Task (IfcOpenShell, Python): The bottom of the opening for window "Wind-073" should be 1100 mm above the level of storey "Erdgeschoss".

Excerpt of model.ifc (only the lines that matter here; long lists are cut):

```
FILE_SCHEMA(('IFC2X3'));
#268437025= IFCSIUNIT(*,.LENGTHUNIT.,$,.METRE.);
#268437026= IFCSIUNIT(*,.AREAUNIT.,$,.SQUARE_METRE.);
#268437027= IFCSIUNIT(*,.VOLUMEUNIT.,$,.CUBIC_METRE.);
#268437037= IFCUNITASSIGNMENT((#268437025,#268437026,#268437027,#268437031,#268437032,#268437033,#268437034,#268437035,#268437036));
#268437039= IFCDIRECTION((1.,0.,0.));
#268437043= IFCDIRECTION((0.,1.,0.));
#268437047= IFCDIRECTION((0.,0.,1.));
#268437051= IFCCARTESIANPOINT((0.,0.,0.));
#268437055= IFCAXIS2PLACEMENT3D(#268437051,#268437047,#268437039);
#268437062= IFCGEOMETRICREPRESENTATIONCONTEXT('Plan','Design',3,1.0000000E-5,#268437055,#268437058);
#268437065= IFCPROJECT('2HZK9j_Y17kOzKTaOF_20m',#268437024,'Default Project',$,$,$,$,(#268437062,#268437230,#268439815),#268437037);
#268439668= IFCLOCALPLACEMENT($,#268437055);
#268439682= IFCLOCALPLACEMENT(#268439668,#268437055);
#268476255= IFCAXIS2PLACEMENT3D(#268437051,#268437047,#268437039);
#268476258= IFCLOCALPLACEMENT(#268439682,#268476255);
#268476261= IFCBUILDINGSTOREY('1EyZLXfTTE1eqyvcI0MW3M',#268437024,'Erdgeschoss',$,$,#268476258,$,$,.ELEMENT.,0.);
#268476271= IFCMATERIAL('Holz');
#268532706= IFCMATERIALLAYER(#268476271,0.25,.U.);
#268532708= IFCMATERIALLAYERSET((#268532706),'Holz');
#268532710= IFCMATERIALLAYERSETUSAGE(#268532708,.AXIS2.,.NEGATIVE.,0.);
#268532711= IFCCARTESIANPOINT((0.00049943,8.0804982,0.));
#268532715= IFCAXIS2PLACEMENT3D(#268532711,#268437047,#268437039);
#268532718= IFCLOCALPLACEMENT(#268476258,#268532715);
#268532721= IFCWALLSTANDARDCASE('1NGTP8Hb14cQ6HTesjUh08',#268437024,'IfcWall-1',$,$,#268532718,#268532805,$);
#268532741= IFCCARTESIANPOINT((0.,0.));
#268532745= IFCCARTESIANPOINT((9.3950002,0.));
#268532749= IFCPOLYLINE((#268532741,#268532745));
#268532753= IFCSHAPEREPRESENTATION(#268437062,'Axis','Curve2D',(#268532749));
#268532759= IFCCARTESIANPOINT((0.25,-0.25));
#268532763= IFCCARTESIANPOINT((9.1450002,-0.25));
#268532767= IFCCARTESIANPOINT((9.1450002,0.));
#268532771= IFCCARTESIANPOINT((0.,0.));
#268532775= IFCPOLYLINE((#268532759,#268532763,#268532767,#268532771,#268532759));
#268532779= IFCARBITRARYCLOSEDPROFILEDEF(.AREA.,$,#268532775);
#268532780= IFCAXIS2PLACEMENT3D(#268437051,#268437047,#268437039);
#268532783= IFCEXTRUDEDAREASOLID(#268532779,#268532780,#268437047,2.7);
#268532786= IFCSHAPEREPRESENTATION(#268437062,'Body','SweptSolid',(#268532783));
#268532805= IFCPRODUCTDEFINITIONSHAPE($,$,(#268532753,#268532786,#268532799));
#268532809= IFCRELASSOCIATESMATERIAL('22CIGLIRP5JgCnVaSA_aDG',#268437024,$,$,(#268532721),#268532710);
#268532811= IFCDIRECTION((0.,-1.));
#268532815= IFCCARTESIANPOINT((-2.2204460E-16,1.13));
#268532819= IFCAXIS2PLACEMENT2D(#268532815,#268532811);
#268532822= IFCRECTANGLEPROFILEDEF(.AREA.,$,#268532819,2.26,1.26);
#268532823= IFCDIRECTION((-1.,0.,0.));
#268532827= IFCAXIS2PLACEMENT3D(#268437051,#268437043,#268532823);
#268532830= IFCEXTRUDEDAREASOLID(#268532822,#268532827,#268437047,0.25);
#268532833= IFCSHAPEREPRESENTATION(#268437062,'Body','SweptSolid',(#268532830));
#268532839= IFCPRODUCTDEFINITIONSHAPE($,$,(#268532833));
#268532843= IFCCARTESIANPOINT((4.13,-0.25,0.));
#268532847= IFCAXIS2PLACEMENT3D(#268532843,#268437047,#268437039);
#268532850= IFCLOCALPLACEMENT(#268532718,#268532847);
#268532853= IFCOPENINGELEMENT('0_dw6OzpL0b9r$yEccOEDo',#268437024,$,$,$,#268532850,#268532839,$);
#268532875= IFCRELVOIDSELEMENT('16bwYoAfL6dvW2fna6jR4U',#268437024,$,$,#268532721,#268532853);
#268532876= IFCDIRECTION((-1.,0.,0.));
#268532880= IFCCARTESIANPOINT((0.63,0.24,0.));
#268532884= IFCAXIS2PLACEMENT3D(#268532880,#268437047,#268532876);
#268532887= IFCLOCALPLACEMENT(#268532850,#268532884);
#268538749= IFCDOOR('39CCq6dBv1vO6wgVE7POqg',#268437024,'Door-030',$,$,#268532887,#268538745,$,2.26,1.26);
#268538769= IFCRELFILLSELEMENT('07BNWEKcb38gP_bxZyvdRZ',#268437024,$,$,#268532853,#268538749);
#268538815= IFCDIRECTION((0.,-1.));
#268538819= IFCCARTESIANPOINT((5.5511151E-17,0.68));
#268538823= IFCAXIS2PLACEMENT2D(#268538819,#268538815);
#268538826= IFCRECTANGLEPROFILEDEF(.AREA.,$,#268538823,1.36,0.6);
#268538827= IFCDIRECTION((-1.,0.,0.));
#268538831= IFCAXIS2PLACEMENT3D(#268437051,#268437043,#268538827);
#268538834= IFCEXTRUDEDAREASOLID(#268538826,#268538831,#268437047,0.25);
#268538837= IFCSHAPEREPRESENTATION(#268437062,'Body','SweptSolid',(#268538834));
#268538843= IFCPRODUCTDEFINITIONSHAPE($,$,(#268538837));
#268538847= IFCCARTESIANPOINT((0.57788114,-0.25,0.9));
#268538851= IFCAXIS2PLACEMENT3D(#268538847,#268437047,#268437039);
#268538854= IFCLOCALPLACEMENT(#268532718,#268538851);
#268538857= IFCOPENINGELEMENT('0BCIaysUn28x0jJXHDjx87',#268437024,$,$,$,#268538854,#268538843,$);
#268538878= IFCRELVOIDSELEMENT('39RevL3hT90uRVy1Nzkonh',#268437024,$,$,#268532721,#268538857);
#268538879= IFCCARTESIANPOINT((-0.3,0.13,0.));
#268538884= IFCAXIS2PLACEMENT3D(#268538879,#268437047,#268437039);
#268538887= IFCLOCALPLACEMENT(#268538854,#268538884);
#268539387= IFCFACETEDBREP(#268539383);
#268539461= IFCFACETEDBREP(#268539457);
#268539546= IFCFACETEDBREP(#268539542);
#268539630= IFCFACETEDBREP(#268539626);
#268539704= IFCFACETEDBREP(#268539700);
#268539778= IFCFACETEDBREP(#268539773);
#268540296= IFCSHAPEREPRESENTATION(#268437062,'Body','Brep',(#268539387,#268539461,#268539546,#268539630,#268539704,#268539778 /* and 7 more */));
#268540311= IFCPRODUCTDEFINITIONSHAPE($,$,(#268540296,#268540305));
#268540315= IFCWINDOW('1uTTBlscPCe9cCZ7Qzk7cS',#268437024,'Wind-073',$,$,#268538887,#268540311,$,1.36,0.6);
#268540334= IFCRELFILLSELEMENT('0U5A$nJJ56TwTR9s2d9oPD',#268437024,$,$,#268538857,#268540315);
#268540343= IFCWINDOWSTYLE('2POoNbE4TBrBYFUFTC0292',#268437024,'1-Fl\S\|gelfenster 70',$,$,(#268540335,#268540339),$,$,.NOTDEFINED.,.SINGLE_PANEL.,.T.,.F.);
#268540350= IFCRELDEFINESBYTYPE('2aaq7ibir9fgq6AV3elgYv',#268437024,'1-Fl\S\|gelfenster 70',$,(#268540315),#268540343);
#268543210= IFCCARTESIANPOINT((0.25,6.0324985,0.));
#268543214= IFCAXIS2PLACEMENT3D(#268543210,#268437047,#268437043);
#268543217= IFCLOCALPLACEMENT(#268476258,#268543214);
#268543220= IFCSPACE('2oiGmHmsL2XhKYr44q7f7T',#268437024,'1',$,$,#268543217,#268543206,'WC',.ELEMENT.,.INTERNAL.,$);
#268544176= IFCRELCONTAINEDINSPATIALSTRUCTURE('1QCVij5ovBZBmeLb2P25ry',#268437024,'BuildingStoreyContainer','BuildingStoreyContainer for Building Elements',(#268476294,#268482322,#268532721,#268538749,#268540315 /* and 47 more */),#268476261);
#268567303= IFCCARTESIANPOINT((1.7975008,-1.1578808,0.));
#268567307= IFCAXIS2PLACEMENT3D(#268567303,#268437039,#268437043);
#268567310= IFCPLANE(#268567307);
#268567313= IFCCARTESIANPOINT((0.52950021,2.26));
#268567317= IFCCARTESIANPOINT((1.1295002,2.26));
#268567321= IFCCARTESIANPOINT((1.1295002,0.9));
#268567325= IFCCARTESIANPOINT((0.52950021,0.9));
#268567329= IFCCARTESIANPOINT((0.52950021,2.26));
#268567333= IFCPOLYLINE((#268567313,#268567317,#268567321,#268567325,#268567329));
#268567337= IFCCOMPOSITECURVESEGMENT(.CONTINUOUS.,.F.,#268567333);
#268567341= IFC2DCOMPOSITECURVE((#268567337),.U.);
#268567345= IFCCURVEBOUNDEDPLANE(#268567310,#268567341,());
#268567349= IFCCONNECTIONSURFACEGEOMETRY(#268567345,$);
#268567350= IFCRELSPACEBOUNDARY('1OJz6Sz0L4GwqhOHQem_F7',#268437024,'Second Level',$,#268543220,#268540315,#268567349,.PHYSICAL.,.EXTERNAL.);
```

```python
import numpy as np
import ifcopenshell
import ifcopenshell.api.geometry
import ifcopenshell.geom
import ifcopenshell.util.element
import ifcopenshell.util.placement
import ifcopenshell.util.shape
import ifcopenshell.util.unit

model = ifcopenshell.open("model.ifc")
unit_scale = ifcopenshell.util.unit.calculate_unit_scale(model)

window = model.by_guid("1uTTBlscPCe9cCZ7Qzk7cS")
opening = window.FillsVoids[0].RelatingOpeningElement
storey = ifcopenshell.util.element.get_container(window, ifc_class="IfcBuildingStorey")
level = ifcopenshell.util.placement.get_local_placement(storey.ObjectPlacement)[2, 3]

# The opening's origin need not be at the sill, so measure its lowest point.
shape = ifcopenshell.geom.create_shape(ifcopenshell.geom.settings(), opening)
bottom = ifcopenshell.util.shape.get_shape_bottom_elevation(shape, shape.geometry) / unit_scale
dz = level + 1.1 - bottom

shift = np.array([0.0, 0.0, dz])
# The window is placed relative to its opening, so it follows when the opening moves.
matrix = ifcopenshell.util.placement.get_local_placement(opening.ObjectPlacement)
matrix[:3, 3] += shift
ifcopenshell.api.geometry.edit_object_placement(
    model, product=opening, matrix=matrix, is_si=False, should_transform_children=True
)

# Space boundary surfaces are stored in each space's coordinates; move them too.
for rel in window.ProvidesBoundaries:
    if not rel.ConnectionGeometry:
        continue
    surface = rel.ConnectionGeometry.SurfaceOnRelatingElement.BasisSurface
    space_matrix = ifcopenshell.util.placement.get_local_placement(rel.RelatingSpace.ObjectPlacement)
    point = np.array(surface.Position.Location.Coordinates) + space_matrix[:3, :3].T @ shift
    surface.Position = model.createIfcAxis2Placement3D(
        model.createIfcCartesianPoint(point.tolist()), surface.Position.Axis, surface.Position.RefDirection
    )

print(f"moved by {dz * unit_scale:+.3f} m")

model.write("model-out.ifc")
```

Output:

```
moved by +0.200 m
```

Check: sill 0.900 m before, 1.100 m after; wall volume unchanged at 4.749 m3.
